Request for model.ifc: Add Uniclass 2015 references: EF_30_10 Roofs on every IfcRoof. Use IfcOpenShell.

First a look at what the model holds.

```python
import ifcopenshell

model = ifcopenshell.open("model.ifc")
print(model.schema)
print("classifications:", [c.Name for c in model.by_type("IfcClassification")])
for ifc_class in ("IfcDoor", "IfcRoof", "IfcStair", "IfcWall", "IfcWindow"):
    print(ifc_class, len(model.by_type(ifc_class)))
```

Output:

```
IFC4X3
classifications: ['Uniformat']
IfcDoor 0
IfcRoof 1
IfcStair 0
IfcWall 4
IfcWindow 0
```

```python
import ifcopenshell
import ifcopenshell.api.classification

model = ifcopenshell.open("model.ifc")

system = ifcopenshell.api.classification.add_classification(model, classification="Uniclass 2015")

codes = {
    "IfcRoof": ("EF_30_10", "Roofs"),
}
for ifc_class, (code, name) in codes.items():
    products = model.by_type(ifc_class)
    ifcopenshell.api.classification.add_reference(
        model, products=products, classification=system, identification=code, name=name
    )
    print(code, len(products))

model.write("model-out.ifc")
```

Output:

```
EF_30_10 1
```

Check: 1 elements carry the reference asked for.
